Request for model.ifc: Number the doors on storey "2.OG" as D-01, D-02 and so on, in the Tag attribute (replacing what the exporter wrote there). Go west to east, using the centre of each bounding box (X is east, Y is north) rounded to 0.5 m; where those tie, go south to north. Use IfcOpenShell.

First a look at what the model holds.

```python
import ifcopenshell
import ifcopenshell.util.element
import ifcopenshell.util.placement

model = ifcopenshell.open("model.ifc")
print(model.schema)
storey = next(s for s in model.by_type("IfcBuildingStorey") if s.Name == "2.OG")
doors = [e for e in ifcopenshell.util.element.get_decomposition(storey) if e.is_a("IfcDoor")]
for e in sorted(doors, key=lambda e: e.id()):
    origin = ifcopenshell.util.placement.get_local_placement(e.ObjectPlacement)[:3, 3]
    print(e.id(), e.Tag, e.Name, origin.round(2) + 0.0, sep=" | ")
```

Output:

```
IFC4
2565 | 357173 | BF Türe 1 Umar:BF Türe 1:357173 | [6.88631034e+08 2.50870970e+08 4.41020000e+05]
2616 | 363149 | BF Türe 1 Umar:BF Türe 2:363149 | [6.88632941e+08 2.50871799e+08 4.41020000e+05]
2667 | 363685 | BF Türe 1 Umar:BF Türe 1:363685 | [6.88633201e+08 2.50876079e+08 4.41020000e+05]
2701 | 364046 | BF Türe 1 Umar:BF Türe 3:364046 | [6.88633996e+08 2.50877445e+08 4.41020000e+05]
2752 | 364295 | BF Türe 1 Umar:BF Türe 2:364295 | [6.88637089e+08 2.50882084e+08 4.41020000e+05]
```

```python
import ifcopenshell
import ifcopenshell.geom
import ifcopenshell.util.element
import ifcopenshell.util.shape

model = ifcopenshell.open("model.ifc")
settings = ifcopenshell.geom.settings()
settings.set("use-world-coords", True)


def centre(element):
    shape = ifcopenshell.geom.create_shape(settings, element)
    return ifcopenshell.util.shape.get_bbox_centroid(shape.geometry)


storey = next(s for s in model.by_type("IfcBuildingStorey") if s.Name == "2.OG")
doors = [e for e in ifcopenshell.util.element.get_decomposition(storey) if e.is_a("IfcDoor")]

# Insertion points can sit at a corner or the storey origin, so sort by the geometry (in metres).
centres = {e: centre(e) for e in doors}
doors.sort(key=lambda e: (round(centres[e][0] / 0.5), centres[e][1]))

for i, e in enumerate(doors, start=1):
    number = f"D-{i:02d}"
    e.Tag = number
    print(e.id(), number)

model.write("model-out.ifc")
```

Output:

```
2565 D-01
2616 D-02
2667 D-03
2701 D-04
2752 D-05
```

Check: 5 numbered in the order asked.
